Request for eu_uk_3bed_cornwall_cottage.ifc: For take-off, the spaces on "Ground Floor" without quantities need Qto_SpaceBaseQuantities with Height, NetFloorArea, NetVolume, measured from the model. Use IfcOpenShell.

First a look at what the model holds.

```python
import ifcopenshell
import ifcopenshell.util.element
import ifcopenshell.util.unit

model = ifcopenshell.open("eu_uk_3bed_cornwall_cottage.ifc")
print(model.schema)
for unit_type in ("LENGTHUNIT", "AREAUNIT", "VOLUMEUNIT"):
    print(unit_type, ifcopenshell.util.unit.calculate_unit_scale(model, unit_type))
storey = next(s for s in model.by_type("IfcBuildingStorey") if s.Name == "Ground Floor")
spaces = [e for e in ifcopenshell.util.element.get_decomposition(storey) if e.is_a("IfcSpace")]
for e in sorted(spaces, key=lambda e: e.id()):
    print(e.id(), e.is_a(), e.Name, list(ifcopenshell.util.element.get_psets(e, qtos_only=True)), sep=" | ")
```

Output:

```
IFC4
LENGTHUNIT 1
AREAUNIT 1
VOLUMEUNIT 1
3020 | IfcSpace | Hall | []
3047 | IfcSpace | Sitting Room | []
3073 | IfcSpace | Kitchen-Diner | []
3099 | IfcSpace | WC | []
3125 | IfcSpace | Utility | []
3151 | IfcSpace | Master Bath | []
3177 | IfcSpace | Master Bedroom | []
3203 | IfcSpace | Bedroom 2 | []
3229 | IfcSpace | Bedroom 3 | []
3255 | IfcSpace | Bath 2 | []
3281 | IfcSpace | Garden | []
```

```python
import ifcopenshell
import ifcopenshell.api.pset
import ifcopenshell.geom
import ifcopenshell.util.element
import ifcopenshell.util.shape
import ifcopenshell.util.unit

model = ifcopenshell.open("eu_uk_3bed_cornwall_cottage.ifc")
unit_scale = ifcopenshell.util.unit.calculate_unit_scale(model)
area_scale = ifcopenshell.util.unit.calculate_unit_scale(model, "AREAUNIT")
volume_scale = ifcopenshell.util.unit.calculate_unit_scale(model, "VOLUMEUNIT")
settings = ifcopenshell.geom.settings()

storey = next(s for s in model.by_type("IfcBuildingStorey") if s.Name == "Ground Floor")
spaces = [e for e in ifcopenshell.util.element.get_decomposition(storey) if e.is_a("IfcSpace")]

for e in sorted(spaces, key=lambda e: e.id()):
    if ifcopenshell.util.element.get_psets(e, qtos_only=True, should_inherit=False):
        continue
    # Geometry comes back in metres, in the element's own axes.
    shape = ifcopenshell.geom.create_shape(settings, e)
    values = {
        "Height": ifcopenshell.util.shape.get_z(shape.geometry) / unit_scale,
        "NetFloorArea": ifcopenshell.util.shape.get_footprint_area(shape.geometry) / area_scale,
        "NetVolume": ifcopenshell.util.shape.get_volume(shape.geometry) / volume_scale,
    }
    qto = ifcopenshell.api.pset.add_qto(model, product=e, name="Qto_SpaceBaseQuantities")
    ifcopenshell.api.pset.edit_qto(model, qto=qto, properties=values)
    print(e.id(), {k: round(v, 3) for k, v in values.items()})

model.write("eu_uk_3bed_cornwall_cottage_rev.ifc")
```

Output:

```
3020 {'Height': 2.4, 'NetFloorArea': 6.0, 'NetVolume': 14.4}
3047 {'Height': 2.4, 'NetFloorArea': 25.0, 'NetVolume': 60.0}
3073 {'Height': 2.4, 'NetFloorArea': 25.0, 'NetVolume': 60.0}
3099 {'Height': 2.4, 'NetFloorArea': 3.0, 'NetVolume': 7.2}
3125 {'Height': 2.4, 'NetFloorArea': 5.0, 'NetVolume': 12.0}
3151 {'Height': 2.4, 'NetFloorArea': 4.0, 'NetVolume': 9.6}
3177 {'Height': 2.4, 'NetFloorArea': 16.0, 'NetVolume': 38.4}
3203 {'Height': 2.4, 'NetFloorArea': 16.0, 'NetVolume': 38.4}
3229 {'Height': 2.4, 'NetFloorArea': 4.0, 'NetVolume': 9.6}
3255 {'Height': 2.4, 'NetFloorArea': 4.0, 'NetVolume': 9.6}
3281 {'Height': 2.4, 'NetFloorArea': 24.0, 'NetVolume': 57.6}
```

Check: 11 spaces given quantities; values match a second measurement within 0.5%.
